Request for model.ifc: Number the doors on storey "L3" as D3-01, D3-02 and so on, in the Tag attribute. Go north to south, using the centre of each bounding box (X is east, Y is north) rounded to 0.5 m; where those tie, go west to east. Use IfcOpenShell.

First a look at what the model holds.

```python
import ifcopenshell
import ifcopenshell.util.element
import ifcopenshell.util.placement

model = ifcopenshell.open("model.ifc")
print(model.schema)
storey = next(s for s in model.by_type("IfcBuildingStorey") if s.Name == "L3")
doors = [e for e in ifcopenshell.util.element.get_decomposition(storey) if e.is_a("IfcDoor")]
for e in sorted(doors, key=lambda e: e.id()):
    origin = ifcopenshell.util.placement.get_local_placement(e.ObjectPlacement)[:3, 3]
    print(e.id(), e.Tag, e.Name, origin.round(2) + 0.0, sep=" | ")
```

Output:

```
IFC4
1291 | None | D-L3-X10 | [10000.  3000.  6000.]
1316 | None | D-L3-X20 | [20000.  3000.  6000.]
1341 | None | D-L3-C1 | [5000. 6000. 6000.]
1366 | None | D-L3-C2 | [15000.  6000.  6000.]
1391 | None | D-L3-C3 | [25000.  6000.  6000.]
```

```python
import ifcopenshell
import ifcopenshell.geom
import ifcopenshell.util.element
import ifcopenshell.util.shape

model = ifcopenshell.open("model.ifc")
settings = ifcopenshell.geom.settings()
settings.set("use-world-coords", True)


def centre(element):
    shape = ifcopenshell.geom.create_shape(settings, element)
    return ifcopenshell.util.shape.get_bbox_centroid(shape.geometry)


storey = next(s for s in model.by_type("IfcBuildingStorey") if s.Name == "L3")
doors = [e for e in ifcopenshell.util.element.get_decomposition(storey) if e.is_a("IfcDoor")]

# Insertion points can sit at a corner or the storey origin, so sort by the geometry (in metres).
centres = {e: centre(e) for e in doors}
doors.sort(key=lambda e: (-round(centres[e][1] / 0.5), centres[e][0]))

for i, e in enumerate(doors, start=1):
    number = f"D3-{i:02d}"
    e.Tag = number
    print(e.id(), number)

model.write("model-out.ifc")
```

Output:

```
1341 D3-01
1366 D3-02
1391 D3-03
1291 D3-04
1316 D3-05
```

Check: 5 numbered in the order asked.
